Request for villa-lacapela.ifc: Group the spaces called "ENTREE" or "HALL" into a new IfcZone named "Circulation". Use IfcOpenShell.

First a look at what the model holds.

```python
import ifcopenshell

model = ifcopenshell.open("villa-lacapela.ifc")
print(model.schema)
seen = {}
for space in model.by_type("IfcSpace"):
    seen[space.LongName] = seen.get(space.LongName, 0) + 1
for name, count in sorted(seen.items(), key=str):
    print(count, "x", name)
print("zones:", [z.Name for z in model.by_type("IfcZone")][:20])
```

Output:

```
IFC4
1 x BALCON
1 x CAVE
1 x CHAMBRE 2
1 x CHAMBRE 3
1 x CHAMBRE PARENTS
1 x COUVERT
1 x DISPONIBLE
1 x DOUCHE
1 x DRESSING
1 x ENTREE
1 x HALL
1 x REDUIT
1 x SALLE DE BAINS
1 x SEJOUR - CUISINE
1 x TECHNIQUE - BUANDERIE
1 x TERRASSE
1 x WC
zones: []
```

```python
import ifcopenshell
import ifcopenshell.api.group
import ifcopenshell.api.root

model = ifcopenshell.open("villa-lacapela.ifc")

names = {"ENTREE", "HALL"}
spaces = [s for s in model.by_type("IfcSpace") if s.LongName in names]

zone = ifcopenshell.api.root.create_entity(model, ifc_class="IfcZone", name="Circulation")
ifcopenshell.api.group.assign_group(model, products=spaces, group=zone)
print(len(spaces), "spaces in", zone.Name)

model.write("villa-lacapela_rev.ifc")
```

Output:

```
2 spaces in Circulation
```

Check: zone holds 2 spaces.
